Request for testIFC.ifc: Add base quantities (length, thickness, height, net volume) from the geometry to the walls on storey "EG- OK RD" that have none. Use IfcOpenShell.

First a look at what the model holds.

```python
import ifcopenshell
import ifcopenshell.util.element
import ifcopenshell.util.unit

model = ifcopenshell.open("testIFC.ifc")
print(model.schema)
for unit_type in ("LENGTHUNIT", "AREAUNIT", "VOLUMEUNIT"):
    print(unit_type, ifcopenshell.util.unit.calculate_unit_scale(model, unit_type))
storey = next(s for s in model.by_type("IfcBuildingStorey") if s.Name == "EG- OK RD")
walls = [e for e in ifcopenshell.util.element.get_decomposition(storey) if e.is_a("IfcWall")]
for e in sorted(walls, key=lambda e: e.id()):
    print(e.id(), e.is_a(), e.Name, list(ifcopenshell.util.element.get_psets(e, qtos_only=True)), sep=" | ")
```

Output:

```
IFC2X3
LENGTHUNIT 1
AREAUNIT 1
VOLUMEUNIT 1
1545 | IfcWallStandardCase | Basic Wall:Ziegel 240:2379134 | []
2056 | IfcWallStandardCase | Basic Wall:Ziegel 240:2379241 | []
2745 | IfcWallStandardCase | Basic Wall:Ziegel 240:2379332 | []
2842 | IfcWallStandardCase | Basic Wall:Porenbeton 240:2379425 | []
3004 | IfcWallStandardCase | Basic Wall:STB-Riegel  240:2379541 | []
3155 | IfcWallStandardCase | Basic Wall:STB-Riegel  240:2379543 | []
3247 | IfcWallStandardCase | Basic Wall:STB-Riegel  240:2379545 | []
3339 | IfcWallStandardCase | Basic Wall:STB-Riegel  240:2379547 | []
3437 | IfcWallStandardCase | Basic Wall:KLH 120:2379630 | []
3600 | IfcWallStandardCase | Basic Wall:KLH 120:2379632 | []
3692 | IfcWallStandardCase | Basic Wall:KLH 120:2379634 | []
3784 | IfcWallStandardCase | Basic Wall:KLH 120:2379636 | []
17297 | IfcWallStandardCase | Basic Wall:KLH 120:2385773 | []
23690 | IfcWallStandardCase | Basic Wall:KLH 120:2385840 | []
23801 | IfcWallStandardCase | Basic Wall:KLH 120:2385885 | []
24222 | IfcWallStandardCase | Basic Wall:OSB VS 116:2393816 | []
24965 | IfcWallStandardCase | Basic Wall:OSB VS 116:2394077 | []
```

```python
import ifcopenshell
import ifcopenshell.api.pset
import ifcopenshell.geom
import ifcopenshell.util.element
import ifcopenshell.util.shape
import ifcopenshell.util.unit

model = ifcopenshell.open("testIFC.ifc")
unit_scale = ifcopenshell.util.unit.calculate_unit_scale(model)
volume_scale = ifcopenshell.util.unit.calculate_unit_scale(model, "VOLUMEUNIT")
settings = ifcopenshell.geom.settings()

storey = next(s for s in model.by_type("IfcBuildingStorey") if s.Name == "EG- OK RD")
walls = [e for e in ifcopenshell.util.element.get_decomposition(storey) if e.is_a("IfcWall")]

for e in sorted(walls, key=lambda e: e.id()):
    if ifcopenshell.util.element.get_psets(e, qtos_only=True, should_inherit=False):
        continue
    # Geometry comes back in metres, in the element's own axes.
    shape = ifcopenshell.geom.create_shape(settings, e)
    values = {
        "Length": ifcopenshell.util.shape.get_x(shape.geometry) / unit_scale,
        "Width": ifcopenshell.util.shape.get_y(shape.geometry) / unit_scale,
        "Height": ifcopenshell.util.shape.get_z(shape.geometry) / unit_scale,
        "NetVolume": ifcopenshell.util.shape.get_volume(shape.geometry) / volume_scale,
    }
    qto = ifcopenshell.api.pset.add_qto(model, product=e, name="BaseQuantities")
    ifcopenshell.api.pset.edit_qto(model, qto=qto, properties=values)
    print(e.id(), {k: round(v, 3) for k, v in values.items()})

model.write("testIFC_edited.ifc")
```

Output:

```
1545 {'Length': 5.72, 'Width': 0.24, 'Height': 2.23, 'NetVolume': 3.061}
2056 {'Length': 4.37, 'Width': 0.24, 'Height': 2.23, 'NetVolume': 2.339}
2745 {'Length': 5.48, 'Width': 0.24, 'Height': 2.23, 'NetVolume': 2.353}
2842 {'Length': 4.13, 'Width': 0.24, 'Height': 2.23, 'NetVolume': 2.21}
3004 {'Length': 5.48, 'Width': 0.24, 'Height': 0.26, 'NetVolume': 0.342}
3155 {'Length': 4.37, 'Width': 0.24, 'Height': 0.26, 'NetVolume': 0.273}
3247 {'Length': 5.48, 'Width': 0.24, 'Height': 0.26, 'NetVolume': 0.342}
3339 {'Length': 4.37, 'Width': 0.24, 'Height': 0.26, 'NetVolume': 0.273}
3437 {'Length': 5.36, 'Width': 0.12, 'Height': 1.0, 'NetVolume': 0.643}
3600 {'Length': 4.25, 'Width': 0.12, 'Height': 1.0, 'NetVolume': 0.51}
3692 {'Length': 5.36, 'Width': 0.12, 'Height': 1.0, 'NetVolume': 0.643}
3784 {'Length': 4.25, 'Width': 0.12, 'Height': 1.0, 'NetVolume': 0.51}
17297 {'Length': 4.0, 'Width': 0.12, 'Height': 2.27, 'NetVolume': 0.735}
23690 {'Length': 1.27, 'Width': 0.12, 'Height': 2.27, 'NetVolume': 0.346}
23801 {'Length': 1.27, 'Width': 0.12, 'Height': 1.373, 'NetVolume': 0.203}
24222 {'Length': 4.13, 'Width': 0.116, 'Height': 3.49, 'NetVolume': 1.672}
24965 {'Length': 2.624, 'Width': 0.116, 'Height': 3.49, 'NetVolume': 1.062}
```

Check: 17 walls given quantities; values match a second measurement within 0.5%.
